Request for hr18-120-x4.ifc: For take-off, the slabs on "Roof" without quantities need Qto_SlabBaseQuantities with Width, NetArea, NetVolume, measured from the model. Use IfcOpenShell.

First a look at what the model holds.

```python
import ifcopenshell
import ifcopenshell.util.element
import ifcopenshell.util.unit

model = ifcopenshell.open("hr18-120-x4.ifc")
print(model.schema)
for unit_type in ("LENGTHUNIT", "AREAUNIT", "VOLUMEUNIT"):
    print(unit_type, ifcopenshell.util.unit.calculate_unit_scale(model, unit_type))
storey = next(s for s in model.by_type("IfcBuildingStorey") if s.Name == "Roof")
slabs = [e for e in ifcopenshell.util.element.get_decomposition(storey) if e.is_a("IfcSlab")]
for e in sorted(slabs, key=lambda e: e.id()):
    print(e.id(), e.is_a(), e.Name, list(ifcopenshell.util.element.get_psets(e, qtos_only=True)), sep=" | ")
```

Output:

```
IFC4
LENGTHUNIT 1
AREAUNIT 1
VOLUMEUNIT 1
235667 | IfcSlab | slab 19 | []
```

```python
import ifcopenshell
import ifcopenshell.api.pset
import ifcopenshell.geom
import ifcopenshell.util.element
import ifcopenshell.util.shape
import ifcopenshell.util.unit

model = ifcopenshell.open("hr18-120-x4.ifc")
unit_scale = ifcopenshell.util.unit.calculate_unit_scale(model)
area_scale = ifcopenshell.util.unit.calculate_unit_scale(model, "AREAUNIT")
volume_scale = ifcopenshell.util.unit.calculate_unit_scale(model, "VOLUMEUNIT")
settings = ifcopenshell.geom.settings()

storey = next(s for s in model.by_type("IfcBuildingStorey") if s.Name == "Roof")
slabs = [e for e in ifcopenshell.util.element.get_decomposition(storey) if e.is_a("IfcSlab")]

for e in sorted(slabs, key=lambda e: e.id()):
    if ifcopenshell.util.element.get_psets(e, qtos_only=True, should_inherit=False):
        continue
    # Geometry comes back in metres, in the element's own axes.
    shape = ifcopenshell.geom.create_shape(settings, e)
    values = {
        "Width": ifcopenshell.util.shape.get_z(shape.geometry) / unit_scale,
        "NetArea": ifcopenshell.util.shape.get_footprint_area(shape.geometry) / area_scale,
        "NetVolume": ifcopenshell.util.shape.get_volume(shape.geometry) / volume_scale,
    }
    qto = ifcopenshell.api.pset.add_qto(model, product=e, name="Qto_SlabBaseQuantities")
    ifcopenshell.api.pset.edit_qto(model, qto=qto, properties=values)
    print(e.id(), {k: round(v, 3) for k, v in values.items()})

model.write("hr18-120-x4_updated.ifc")
```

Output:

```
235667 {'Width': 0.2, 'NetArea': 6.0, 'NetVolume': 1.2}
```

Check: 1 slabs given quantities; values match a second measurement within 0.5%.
